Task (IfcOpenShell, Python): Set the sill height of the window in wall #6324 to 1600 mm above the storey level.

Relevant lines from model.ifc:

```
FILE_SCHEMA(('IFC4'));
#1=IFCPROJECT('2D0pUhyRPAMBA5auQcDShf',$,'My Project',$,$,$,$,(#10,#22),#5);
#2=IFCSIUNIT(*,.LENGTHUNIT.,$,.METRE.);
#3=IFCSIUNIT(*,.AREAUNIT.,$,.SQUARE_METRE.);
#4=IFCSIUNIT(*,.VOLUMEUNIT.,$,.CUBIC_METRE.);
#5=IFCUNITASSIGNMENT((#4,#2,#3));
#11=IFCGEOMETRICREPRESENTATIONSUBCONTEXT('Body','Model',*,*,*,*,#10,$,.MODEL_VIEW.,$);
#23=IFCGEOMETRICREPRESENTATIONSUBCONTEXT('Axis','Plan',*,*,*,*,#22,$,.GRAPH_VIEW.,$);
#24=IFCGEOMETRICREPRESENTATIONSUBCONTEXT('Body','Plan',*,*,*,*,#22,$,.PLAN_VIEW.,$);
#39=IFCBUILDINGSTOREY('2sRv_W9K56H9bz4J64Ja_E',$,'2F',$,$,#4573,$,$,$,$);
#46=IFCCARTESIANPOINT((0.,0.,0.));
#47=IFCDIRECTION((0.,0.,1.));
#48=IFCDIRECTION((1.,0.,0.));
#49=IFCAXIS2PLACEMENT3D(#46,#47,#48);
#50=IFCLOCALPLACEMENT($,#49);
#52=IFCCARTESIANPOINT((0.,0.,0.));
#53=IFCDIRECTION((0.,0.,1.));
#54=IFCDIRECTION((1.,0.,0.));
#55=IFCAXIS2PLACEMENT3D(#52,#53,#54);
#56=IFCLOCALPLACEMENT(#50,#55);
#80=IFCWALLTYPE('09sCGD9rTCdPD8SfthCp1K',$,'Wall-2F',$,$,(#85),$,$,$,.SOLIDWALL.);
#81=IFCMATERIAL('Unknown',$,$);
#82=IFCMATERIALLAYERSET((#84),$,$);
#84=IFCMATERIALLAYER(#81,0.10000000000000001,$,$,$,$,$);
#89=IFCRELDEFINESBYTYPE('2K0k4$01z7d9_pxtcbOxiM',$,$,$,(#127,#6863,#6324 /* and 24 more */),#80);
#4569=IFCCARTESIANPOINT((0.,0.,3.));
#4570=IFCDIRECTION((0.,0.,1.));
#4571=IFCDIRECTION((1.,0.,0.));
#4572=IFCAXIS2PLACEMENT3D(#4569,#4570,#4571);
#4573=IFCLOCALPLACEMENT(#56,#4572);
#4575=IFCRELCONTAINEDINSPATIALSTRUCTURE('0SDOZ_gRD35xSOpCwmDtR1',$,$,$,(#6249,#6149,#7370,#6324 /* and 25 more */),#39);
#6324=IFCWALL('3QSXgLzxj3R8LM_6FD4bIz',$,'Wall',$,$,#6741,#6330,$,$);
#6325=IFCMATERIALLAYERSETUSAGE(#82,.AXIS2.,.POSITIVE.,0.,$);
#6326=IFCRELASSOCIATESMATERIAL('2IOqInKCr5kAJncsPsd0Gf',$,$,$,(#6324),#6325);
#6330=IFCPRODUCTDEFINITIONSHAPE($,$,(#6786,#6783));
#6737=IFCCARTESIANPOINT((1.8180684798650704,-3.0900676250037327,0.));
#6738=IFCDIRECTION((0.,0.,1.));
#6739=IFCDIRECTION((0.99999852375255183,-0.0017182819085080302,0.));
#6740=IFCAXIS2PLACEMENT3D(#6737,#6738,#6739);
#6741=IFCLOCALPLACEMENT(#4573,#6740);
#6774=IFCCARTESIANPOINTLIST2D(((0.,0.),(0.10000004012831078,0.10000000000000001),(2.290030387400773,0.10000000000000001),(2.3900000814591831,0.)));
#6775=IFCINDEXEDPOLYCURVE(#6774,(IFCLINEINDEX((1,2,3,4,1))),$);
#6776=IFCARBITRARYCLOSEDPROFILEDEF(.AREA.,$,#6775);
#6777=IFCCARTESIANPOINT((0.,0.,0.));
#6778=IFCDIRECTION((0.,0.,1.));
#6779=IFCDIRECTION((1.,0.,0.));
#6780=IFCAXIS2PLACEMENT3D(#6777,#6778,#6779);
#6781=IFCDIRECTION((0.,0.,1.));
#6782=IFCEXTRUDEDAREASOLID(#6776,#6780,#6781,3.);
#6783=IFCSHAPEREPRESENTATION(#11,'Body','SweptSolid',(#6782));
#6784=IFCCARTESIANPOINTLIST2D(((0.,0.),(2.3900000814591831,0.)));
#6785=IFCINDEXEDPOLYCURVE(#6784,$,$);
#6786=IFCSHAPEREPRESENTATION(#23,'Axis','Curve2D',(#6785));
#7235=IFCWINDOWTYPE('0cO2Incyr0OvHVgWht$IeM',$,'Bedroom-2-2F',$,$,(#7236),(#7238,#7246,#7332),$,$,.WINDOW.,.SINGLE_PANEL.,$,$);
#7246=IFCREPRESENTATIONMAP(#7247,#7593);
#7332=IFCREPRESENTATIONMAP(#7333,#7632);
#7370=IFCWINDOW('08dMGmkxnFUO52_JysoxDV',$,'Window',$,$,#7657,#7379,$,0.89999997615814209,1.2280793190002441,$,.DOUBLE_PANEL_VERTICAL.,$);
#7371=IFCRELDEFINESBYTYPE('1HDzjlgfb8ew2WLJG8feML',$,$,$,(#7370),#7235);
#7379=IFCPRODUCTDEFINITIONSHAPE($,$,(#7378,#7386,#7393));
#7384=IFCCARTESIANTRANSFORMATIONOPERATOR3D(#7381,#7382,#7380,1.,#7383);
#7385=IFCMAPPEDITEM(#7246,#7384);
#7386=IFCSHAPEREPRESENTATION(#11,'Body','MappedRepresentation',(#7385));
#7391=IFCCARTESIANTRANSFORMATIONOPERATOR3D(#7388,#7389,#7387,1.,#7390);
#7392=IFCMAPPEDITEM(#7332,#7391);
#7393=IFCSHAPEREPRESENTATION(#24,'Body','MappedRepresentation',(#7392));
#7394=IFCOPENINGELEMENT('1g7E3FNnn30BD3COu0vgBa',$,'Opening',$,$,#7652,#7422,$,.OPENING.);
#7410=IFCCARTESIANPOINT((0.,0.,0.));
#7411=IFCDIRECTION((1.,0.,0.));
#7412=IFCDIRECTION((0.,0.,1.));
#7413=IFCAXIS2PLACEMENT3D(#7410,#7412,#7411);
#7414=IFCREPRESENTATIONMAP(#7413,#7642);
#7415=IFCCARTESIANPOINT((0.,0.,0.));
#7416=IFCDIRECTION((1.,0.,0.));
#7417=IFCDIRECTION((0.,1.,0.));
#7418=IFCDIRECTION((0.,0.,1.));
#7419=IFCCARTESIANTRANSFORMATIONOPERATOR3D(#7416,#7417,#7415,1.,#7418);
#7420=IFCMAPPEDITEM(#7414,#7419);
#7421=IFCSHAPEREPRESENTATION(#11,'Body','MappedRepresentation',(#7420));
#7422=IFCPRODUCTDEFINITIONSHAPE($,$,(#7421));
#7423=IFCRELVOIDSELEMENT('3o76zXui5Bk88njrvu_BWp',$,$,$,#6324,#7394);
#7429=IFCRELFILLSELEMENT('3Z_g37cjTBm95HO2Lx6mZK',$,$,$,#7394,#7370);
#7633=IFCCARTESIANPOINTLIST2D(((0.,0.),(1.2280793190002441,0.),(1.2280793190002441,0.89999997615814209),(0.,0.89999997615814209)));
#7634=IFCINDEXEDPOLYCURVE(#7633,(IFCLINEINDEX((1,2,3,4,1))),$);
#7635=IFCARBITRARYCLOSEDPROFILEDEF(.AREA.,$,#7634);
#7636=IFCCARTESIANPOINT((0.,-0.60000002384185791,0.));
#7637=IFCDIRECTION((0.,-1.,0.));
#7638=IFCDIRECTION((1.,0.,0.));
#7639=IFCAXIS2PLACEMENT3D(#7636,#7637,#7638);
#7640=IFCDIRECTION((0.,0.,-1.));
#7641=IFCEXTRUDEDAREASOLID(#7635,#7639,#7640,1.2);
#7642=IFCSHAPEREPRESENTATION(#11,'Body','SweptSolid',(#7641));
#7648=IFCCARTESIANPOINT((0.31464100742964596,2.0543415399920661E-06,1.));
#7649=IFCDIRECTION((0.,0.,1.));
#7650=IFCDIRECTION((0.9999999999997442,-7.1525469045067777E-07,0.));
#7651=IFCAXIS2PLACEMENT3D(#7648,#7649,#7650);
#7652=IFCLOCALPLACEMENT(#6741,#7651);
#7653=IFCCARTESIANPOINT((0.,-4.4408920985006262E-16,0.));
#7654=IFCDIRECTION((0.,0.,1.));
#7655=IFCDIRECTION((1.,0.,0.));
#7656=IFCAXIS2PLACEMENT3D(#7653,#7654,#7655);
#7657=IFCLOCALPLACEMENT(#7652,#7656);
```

```python
import numpy as np
import ifcopenshell
import ifcopenshell.api.geometry
import ifcopenshell.geom
import ifcopenshell.util.element
import ifcopenshell.util.placement
import ifcopenshell.util.shape
import ifcopenshell.util.unit

model = ifcopenshell.open("model.ifc")
unit_scale = ifcopenshell.util.unit.calculate_unit_scale(model)

window = model.by_guid("08dMGmkxnFUO52_JysoxDV")
opening = window.FillsVoids[0].RelatingOpeningElement
storey = ifcopenshell.util.element.get_container(window, ifc_class="IfcBuildingStorey")
level = ifcopenshell.util.placement.get_local_placement(storey.ObjectPlacement)[2, 3]

# The opening's origin need not be at the sill, so measure its lowest point.
shape = ifcopenshell.geom.create_shape(ifcopenshell.geom.settings(), opening)
bottom = ifcopenshell.util.shape.get_shape_bottom_elevation(shape, shape.geometry) / unit_scale
dz = level + 1.6 / unit_scale - bottom

shift = np.array([0.0, 0.0, dz])
# The window is placed relative to its opening, so it follows when the opening moves.
matrix = ifcopenshell.util.placement.get_local_placement(opening.ObjectPlacement)
matrix[:3, 3] += shift
ifcopenshell.api.geometry.edit_object_placement(
    model, product=opening, matrix=matrix, is_si=False, should_transform_children=True
)

print(f"moved by {dz * unit_scale:+.3f} m")

model.write("model_v2.ifc")
```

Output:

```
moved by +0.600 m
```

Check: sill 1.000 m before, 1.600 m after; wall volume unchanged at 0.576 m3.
